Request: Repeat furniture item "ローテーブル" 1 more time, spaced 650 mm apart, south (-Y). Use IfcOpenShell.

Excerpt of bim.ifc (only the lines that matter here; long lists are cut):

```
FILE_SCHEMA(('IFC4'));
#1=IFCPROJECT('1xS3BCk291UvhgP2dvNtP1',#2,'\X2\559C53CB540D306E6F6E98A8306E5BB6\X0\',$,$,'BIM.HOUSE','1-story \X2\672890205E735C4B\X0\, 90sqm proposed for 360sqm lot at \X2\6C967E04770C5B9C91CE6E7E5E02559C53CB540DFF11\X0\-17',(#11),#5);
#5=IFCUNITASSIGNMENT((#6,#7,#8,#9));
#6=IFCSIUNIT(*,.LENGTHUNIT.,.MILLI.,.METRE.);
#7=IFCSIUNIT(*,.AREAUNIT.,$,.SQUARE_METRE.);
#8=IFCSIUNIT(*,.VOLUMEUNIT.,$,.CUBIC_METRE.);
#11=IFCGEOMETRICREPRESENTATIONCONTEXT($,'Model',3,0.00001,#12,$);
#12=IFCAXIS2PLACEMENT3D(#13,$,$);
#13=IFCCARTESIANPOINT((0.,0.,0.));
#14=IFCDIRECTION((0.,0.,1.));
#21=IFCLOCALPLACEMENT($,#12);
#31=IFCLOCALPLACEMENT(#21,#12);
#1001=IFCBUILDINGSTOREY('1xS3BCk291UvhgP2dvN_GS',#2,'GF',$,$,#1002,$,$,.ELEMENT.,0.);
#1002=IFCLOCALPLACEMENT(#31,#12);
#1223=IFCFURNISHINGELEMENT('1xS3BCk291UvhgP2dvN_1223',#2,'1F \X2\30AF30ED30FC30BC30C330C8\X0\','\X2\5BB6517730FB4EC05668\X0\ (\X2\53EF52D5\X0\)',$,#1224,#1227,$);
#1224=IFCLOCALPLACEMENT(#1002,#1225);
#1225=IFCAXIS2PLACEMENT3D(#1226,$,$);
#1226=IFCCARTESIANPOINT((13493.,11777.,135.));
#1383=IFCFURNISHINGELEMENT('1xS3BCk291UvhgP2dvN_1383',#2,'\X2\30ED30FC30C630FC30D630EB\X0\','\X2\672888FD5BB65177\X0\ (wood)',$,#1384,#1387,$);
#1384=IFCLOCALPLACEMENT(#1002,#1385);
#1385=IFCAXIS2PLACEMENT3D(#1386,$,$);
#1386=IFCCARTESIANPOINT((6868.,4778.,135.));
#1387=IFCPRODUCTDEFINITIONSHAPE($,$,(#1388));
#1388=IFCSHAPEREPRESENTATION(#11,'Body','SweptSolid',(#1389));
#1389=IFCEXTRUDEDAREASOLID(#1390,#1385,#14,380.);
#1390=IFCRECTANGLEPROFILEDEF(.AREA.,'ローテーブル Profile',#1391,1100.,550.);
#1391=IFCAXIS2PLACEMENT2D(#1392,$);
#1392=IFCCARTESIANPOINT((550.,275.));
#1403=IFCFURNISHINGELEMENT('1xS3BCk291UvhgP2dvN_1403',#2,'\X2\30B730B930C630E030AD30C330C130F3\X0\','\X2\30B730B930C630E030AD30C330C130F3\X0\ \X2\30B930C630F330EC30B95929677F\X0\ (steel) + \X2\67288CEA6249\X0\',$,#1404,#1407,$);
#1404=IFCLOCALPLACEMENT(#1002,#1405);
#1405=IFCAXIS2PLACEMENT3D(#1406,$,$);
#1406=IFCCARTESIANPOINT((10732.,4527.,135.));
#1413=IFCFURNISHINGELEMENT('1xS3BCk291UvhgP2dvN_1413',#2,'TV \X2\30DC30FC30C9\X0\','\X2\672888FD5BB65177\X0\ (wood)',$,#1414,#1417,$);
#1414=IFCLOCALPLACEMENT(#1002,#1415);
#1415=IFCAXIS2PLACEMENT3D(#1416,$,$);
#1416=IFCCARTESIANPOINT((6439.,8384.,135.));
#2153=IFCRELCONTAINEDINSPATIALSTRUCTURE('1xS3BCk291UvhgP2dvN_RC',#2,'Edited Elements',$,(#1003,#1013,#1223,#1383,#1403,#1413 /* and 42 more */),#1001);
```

```python
import numpy as np
import ifcopenshell
import ifcopenshell.api.geometry
import ifcopenshell.api.root
import ifcopenshell.util.element
import ifcopenshell.util.placement
import ifcopenshell.util.unit

model = ifcopenshell.open("bim.ifc")
unit_scale = ifcopenshell.util.unit.calculate_unit_scale(model)


def reuse_history(source, copy):
    """copy_class also copies each property set's owner history, people and application; keep the originals."""
    for rel in copy.IsDefinedBy:
        if rel.is_a("IfcRelDefinesByProperties") and (history := rel.RelatingPropertyDefinition.OwnerHistory):
            rel.RelatingPropertyDefinition.OwnerHistory = source.OwnerHistory
            ifcopenshell.util.element.remove_deep2(model, history)


source = model.by_guid("1xS3BCk291UvhgP2dvN_1383")
base = ifcopenshell.util.placement.get_local_placement(source.ObjectPlacement)
step = np.array([0.0, -1.0, 0.0]) * 0.65 / unit_scale

for i in range(1, 2):
    copy = ifcopenshell.api.root.copy_class(model, product=source)
    copy.Representation = ifcopenshell.util.element.copy_deep(
        model, source.Representation, exclude=["IfcGeometricRepresentationContext", "IfcRepresentationMap"]
    )
    reuse_history(source, copy)
    matrix = base.copy()
    matrix[:3, 3] += i * step
    print("added at", matrix[:3, 3].round(3) + 0.0)
    ifcopenshell.api.geometry.edit_object_placement(model, product=copy, matrix=matrix, is_si=False)

model.write("bim_v2.ifc")
```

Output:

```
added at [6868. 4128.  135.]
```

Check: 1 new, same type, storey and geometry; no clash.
